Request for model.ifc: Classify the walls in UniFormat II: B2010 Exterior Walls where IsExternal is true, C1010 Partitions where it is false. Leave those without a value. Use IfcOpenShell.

First a look at what the model holds.

```python
import ifcopenshell
import ifcopenshell.util.element

model = ifcopenshell.open("model.ifc")
print(model.schema)
print("classifications:", [c.Name for c in model.by_type("IfcClassification")])
values = [ifcopenshell.util.element.get_pset(e, "Pset_WallCommon", "IsExternal") for e in model.by_type("IfcWall")]
for value in (True, False, None):
    print("IsExternal", value, values.count(value))
```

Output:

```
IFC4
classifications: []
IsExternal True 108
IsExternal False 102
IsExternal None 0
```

```python
import ifcopenshell
import ifcopenshell.api.classification
import ifcopenshell.util.element

model = ifcopenshell.open("model.ifc")

system = ifcopenshell.api.classification.add_classification(model, classification="UniFormat II")

walls = model.by_type("IfcWall")
external = {e: ifcopenshell.util.element.get_pset(e, "Pset_WallCommon", "IsExternal") for e in walls}
for flag, code, name in ((True, "B2010", "Exterior Walls"), (False, "C1010", "Partitions")):
    products = [e for e in walls if external[e] is flag]
    ifcopenshell.api.classification.add_reference(
        model, products=products, classification=system, identification=code, name=name
    )
    print(code, len(products))

model.write("model_rev.ifc")
```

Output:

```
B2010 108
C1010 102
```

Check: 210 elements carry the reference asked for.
